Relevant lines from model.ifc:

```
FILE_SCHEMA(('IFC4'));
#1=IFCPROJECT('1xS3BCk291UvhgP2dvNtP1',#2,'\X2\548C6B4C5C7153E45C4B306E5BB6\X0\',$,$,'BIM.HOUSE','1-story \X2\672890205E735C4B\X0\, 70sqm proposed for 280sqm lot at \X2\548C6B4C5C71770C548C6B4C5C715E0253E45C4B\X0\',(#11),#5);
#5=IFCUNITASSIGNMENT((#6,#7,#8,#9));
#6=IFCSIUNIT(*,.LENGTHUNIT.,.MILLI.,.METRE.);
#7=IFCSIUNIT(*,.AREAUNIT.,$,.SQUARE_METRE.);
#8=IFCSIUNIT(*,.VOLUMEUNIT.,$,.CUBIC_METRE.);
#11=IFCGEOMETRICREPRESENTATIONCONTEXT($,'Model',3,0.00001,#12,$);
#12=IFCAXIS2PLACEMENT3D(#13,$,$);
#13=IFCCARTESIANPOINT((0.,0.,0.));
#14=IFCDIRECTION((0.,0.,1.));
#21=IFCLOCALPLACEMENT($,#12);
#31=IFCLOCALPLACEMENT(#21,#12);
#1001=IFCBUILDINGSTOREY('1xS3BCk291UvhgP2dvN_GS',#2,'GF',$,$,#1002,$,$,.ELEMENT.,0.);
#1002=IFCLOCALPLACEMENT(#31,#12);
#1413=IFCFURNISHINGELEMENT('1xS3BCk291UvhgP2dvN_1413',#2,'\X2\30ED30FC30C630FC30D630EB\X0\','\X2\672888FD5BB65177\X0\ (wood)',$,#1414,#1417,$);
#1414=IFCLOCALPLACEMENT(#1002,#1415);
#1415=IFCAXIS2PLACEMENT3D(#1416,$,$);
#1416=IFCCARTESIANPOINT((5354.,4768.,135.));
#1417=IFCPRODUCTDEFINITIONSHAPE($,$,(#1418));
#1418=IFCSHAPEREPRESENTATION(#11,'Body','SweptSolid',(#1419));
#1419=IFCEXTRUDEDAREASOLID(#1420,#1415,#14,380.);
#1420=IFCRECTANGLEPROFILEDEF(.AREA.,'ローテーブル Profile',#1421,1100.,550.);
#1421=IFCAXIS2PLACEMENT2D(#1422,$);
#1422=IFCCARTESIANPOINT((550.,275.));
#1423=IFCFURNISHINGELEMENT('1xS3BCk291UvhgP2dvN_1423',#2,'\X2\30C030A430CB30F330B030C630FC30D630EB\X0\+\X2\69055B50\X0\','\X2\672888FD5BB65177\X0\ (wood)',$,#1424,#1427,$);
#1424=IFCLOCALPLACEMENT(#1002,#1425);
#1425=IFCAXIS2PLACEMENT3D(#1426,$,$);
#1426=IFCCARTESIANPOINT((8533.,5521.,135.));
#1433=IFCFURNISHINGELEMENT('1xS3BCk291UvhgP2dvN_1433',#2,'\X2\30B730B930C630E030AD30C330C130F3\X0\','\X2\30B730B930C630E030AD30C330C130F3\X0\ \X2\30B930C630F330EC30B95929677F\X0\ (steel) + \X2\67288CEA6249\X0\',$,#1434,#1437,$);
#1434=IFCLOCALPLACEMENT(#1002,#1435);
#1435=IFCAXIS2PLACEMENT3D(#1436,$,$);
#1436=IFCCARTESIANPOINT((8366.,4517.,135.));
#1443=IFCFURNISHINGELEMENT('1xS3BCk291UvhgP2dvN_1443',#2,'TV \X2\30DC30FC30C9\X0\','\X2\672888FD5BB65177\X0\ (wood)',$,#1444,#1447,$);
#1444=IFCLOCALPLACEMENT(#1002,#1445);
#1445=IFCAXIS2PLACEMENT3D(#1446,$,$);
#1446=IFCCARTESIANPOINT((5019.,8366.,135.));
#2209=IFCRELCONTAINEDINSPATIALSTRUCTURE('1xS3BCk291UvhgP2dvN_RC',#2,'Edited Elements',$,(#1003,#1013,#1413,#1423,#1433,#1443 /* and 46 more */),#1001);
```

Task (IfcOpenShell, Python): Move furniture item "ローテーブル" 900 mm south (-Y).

```python
import ifcopenshell
import ifcopenshell.api.geometry
import ifcopenshell.util.placement
import ifcopenshell.util.unit

model = ifcopenshell.open("model.ifc")
unit_scale = ifcopenshell.util.unit.calculate_unit_scale(model)

item = model.by_id(1413)
matrix = ifcopenshell.util.placement.get_local_placement(item.ObjectPlacement)
matrix[1, 3] -= 0.9 / unit_scale
ifcopenshell.api.geometry.edit_object_placement(model, product=item, matrix=matrix, is_si=False)

print(ifcopenshell.util.placement.get_local_placement(item.ObjectPlacement).round(3) + 0.0)

model.write("model_updated.ifc")
```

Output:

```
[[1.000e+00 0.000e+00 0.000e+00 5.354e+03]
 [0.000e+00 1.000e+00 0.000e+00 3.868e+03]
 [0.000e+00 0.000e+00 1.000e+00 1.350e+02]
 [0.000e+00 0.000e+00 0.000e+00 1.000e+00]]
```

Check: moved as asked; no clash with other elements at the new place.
